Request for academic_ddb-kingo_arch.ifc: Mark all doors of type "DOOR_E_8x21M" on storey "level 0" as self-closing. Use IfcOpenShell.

First a look at what the model holds.

```python
import ifcopenshell
import ifcopenshell.util.element

model = ifcopenshell.open("academic_ddb-kingo_arch.ifc")
print(model.schema)
storey = next(s for s in model.by_type("IfcBuildingStorey") if s.Name == "level 0")
doors = [e for e in ifcopenshell.util.element.get_decomposition(storey) if e.is_a("IfcDoor")]
seen = {}
for e in doors:
    element_type = ifcopenshell.util.element.get_type(e)
    key = (element_type.Name if element_type != e and element_type else None, ifcopenshell.util.element.get_pset(e, "Pset_DoorCommon", "SelfClosing"))
    seen[key] = seen.get(key, 0) + 1
for (name, value), count in sorted(seen.items(), key=str):
    print(count, "x", name, "|", value)
```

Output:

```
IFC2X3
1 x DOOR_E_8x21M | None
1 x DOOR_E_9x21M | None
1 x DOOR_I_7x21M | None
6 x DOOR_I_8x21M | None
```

```python
import ifcopenshell
import ifcopenshell.api.pset
import ifcopenshell.util.element

model = ifcopenshell.open("academic_ddb-kingo_arch.ifc")

storey = next(s for s in model.by_type("IfcBuildingStorey") if s.Name == "level 0")
doors = [e for e in ifcopenshell.util.element.get_decomposition(storey) if e.is_a("IfcDoor")]

count = 0
for e in doors:
    element_type = ifcopenshell.util.element.get_type(e)
    if element_type in (None, e) or element_type.Name != "DOOR_E_8x21M":
        continue
    # add_pset returns the element's existing set when there is one.
    pset = ifcopenshell.api.pset.add_pset(model, product=e, name="Pset_DoorCommon")
    ifcopenshell.api.pset.edit_pset(model, pset=pset, properties={"SelfClosing": True})
    count += 1

print(count, "doors updated")

model.write("academic_ddb-kingo_arch_v2.ifc")
```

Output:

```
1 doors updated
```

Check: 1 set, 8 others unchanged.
